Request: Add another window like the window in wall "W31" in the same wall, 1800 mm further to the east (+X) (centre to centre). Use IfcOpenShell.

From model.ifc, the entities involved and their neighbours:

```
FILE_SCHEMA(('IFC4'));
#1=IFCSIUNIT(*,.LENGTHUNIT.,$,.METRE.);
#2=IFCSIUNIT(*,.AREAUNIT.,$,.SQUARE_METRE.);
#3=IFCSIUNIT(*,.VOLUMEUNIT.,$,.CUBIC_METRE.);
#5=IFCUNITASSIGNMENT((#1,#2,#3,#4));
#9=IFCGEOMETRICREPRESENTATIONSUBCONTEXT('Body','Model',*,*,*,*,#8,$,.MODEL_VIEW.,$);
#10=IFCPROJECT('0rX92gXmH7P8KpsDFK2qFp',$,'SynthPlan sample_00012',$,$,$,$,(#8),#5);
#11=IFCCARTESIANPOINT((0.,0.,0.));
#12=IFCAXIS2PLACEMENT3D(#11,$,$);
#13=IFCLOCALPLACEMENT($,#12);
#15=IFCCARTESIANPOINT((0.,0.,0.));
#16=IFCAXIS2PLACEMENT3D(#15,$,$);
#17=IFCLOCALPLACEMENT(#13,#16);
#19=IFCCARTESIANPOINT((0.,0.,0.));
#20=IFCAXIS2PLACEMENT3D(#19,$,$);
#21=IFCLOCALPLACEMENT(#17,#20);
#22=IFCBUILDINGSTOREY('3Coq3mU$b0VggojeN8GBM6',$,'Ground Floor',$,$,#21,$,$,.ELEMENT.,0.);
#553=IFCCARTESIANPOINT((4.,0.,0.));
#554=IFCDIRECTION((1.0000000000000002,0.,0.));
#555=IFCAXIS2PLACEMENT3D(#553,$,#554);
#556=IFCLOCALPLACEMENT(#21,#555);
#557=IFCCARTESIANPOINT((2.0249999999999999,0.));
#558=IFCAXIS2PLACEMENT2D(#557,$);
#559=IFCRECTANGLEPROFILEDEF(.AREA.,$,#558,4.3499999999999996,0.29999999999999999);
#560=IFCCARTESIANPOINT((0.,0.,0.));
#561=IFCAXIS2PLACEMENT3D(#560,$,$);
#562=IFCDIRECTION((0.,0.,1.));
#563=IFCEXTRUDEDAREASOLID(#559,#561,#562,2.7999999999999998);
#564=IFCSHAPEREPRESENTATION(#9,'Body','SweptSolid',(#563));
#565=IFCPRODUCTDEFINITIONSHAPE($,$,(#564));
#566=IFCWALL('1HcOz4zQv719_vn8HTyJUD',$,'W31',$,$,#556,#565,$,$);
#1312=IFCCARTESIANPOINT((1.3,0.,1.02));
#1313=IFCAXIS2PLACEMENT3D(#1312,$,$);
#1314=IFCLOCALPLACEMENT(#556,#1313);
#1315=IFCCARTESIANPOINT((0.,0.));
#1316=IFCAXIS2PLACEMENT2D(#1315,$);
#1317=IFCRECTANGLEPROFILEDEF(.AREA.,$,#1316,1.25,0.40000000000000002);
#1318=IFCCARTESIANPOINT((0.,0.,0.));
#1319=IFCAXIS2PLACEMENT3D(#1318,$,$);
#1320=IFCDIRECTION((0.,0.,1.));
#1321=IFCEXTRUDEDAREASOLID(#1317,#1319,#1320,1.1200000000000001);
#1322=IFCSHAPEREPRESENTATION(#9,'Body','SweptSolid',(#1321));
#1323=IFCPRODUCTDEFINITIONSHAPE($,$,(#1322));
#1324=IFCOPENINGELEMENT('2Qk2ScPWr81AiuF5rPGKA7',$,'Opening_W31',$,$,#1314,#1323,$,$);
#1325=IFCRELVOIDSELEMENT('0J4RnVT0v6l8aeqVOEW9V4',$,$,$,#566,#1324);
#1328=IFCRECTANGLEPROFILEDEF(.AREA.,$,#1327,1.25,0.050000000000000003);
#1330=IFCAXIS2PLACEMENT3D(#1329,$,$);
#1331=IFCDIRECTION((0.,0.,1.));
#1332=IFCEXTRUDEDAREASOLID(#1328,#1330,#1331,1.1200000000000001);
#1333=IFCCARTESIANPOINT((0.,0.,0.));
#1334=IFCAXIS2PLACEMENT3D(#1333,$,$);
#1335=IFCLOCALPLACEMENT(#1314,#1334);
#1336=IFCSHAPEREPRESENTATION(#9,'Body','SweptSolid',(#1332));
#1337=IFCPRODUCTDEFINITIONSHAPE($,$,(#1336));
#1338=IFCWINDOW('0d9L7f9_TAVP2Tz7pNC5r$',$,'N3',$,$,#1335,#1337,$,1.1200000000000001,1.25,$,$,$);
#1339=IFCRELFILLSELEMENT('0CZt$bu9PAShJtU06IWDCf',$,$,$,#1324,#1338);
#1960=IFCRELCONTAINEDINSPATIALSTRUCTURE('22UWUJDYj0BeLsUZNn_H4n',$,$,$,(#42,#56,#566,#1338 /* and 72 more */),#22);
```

```python
import ifcopenshell
import ifcopenshell.api.feature
import ifcopenshell.api.geometry
import ifcopenshell.api.root
import ifcopenshell.geom
import ifcopenshell.util.element
import ifcopenshell.util.placement
import ifcopenshell.util.shape
import ifcopenshell.util.unit

model = ifcopenshell.open("model.ifc")
unit_scale = ifcopenshell.util.unit.calculate_unit_scale(model)
settings = ifcopenshell.geom.settings()


def volume(element):
    """Net volume in cubic metres, openings subtracted."""
    shape = ifcopenshell.geom.create_shape(settings, element)
    return ifcopenshell.util.shape.get_volume(shape.geometry)


window = model.by_id(1338)
opening = window.FillsVoids[0].RelatingOpeningElement
wall = opening.VoidsElements[0].RelatingBuildingElement
before = volume(wall)
shift = ifcopenshell.util.placement.get_local_placement(wall.ObjectPlacement)[:3, 0] * 1.8 / unit_scale

# copy_class copies the void relationship, type, container and properties, but no geometry.
new_opening = ifcopenshell.api.root.copy_class(model, product=opening)
new_opening.Representation = ifcopenshell.util.element.copy_deep(
    model, opening.Representation, exclude=["IfcGeometricRepresentationContext", "IfcRepresentationMap"]
)
new_window = ifcopenshell.api.root.copy_class(model, product=window)
new_window.Representation = ifcopenshell.util.element.copy_deep(
    model, window.Representation, exclude=["IfcGeometricRepresentationContext", "IfcRepresentationMap"]
)
ifcopenshell.api.feature.add_filling(model, opening=new_opening, element=new_window)

for old, new in ((opening, new_opening), (window, new_window)):
    matrix = ifcopenshell.util.placement.get_local_placement(old.ObjectPlacement)
    matrix[:3, 3] += shift
    ifcopenshell.api.geometry.edit_object_placement(model, product=new, matrix=matrix, is_si=False)

after = volume(wall)

print(f"wall volume {before:.3f} -> {after:.3f} m3")

model.write("model_v2.ifc")
```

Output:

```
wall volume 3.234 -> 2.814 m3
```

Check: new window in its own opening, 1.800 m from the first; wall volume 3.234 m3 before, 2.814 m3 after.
